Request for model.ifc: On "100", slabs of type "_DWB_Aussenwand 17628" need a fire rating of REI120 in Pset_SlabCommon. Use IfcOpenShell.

First a look at what the model holds.

```python
import ifcopenshell
import ifcopenshell.util.element

model = ifcopenshell.open("model.ifc")
print(model.schema)
storey = next(s for s in model.by_type("IfcBuildingStorey") if s.Name == "100")
slabs = [e for e in ifcopenshell.util.element.get_decomposition(storey) if e.is_a("IfcSlab")]
seen = {}
for e in slabs:
    element_type = ifcopenshell.util.element.get_type(e)
    key = (element_type.Name if element_type != e and element_type else None, ifcopenshell.util.element.get_pset(e, "Pset_SlabCommon", "FireRating"))
    seen[key] = seen.get(key, 0) + 1
for (name, value), count in sorted(seen.items(), key=str):
    print(count, "x", name, "|", value)
```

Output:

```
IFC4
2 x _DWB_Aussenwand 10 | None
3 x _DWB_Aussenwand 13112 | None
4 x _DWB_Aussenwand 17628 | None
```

```python
import ifcopenshell
import ifcopenshell.api.pset
import ifcopenshell.util.element

model = ifcopenshell.open("model.ifc")

storey = next(s for s in model.by_type("IfcBuildingStorey") if s.Name == "100")
slabs = [e for e in ifcopenshell.util.element.get_decomposition(storey) if e.is_a("IfcSlab")]

count = 0
for e in slabs:
    element_type = ifcopenshell.util.element.get_type(e)
    if element_type in (None, e) or element_type.Name != "_DWB_Aussenwand 17628":
        continue
    # add_pset returns the element's existing set when there is one.
    pset = ifcopenshell.api.pset.add_pset(model, product=e, name="Pset_SlabCommon")
    ifcopenshell.api.pset.edit_pset(model, pset=pset, properties={"FireRating": "REI120"})
    count += 1

print(count, "slabs updated")

model.write("model_updated.ifc")
```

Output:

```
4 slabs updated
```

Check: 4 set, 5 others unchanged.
